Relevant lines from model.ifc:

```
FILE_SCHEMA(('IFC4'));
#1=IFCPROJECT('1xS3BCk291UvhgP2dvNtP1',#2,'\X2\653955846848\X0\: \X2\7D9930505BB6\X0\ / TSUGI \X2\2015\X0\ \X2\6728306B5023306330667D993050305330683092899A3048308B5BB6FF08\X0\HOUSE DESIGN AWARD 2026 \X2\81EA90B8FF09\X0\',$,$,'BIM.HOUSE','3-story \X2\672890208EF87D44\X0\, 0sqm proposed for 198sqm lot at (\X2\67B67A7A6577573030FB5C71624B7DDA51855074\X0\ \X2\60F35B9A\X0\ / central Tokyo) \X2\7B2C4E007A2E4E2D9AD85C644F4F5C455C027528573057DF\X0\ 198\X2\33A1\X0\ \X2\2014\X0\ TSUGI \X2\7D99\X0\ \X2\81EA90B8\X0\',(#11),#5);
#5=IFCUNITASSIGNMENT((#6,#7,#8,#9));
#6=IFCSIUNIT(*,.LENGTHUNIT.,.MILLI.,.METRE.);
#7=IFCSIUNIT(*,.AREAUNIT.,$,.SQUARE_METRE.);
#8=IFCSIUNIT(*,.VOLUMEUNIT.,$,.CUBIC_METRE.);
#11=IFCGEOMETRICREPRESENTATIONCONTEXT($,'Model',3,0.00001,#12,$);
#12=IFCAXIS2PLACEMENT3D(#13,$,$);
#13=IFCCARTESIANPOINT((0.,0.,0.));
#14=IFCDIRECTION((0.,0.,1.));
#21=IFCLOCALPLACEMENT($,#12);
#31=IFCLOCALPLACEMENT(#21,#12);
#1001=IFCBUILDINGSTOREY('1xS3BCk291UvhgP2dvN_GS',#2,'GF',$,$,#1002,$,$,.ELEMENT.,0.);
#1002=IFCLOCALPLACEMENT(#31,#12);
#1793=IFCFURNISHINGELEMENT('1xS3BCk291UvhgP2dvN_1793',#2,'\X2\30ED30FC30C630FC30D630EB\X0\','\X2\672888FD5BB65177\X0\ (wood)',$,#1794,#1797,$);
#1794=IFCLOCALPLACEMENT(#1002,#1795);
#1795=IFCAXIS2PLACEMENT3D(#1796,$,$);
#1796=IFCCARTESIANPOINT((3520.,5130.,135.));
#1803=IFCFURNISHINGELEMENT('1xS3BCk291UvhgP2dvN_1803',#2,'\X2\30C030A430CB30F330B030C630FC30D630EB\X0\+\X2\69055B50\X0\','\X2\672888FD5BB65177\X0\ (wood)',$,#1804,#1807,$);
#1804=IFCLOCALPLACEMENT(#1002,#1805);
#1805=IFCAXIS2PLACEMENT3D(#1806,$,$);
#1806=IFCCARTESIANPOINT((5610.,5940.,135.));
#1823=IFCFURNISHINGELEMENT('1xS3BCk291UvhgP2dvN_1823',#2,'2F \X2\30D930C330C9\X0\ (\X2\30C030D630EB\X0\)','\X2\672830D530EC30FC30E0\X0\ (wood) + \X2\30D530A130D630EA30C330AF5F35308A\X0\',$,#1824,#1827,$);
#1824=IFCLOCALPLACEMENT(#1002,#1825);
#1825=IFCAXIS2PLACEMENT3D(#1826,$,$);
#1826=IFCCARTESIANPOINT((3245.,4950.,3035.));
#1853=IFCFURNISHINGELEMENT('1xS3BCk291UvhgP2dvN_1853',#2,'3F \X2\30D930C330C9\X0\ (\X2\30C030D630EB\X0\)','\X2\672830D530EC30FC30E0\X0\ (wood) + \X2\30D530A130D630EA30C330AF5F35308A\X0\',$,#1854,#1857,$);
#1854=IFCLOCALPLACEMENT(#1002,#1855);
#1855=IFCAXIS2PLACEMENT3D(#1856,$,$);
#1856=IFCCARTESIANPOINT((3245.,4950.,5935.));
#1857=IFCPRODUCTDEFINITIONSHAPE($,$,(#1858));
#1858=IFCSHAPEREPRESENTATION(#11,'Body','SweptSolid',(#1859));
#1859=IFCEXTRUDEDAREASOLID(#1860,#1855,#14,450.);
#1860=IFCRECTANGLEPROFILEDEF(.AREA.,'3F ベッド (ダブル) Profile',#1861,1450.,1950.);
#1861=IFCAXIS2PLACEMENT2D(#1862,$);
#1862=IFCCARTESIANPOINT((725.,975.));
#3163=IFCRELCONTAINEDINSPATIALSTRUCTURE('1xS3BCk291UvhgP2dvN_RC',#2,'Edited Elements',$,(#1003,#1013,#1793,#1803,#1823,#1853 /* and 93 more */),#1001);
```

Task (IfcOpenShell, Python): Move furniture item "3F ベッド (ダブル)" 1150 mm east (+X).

```python
import ifcopenshell
import ifcopenshell.api.geometry
import ifcopenshell.util.placement

model = ifcopenshell.open("model.ifc")

item = model.by_guid("1xS3BCk291UvhgP2dvN_1853")
matrix = ifcopenshell.util.placement.get_local_placement(item.ObjectPlacement)
matrix[0, 3] += 1150.0
ifcopenshell.api.geometry.edit_object_placement(model, product=item, matrix=matrix, is_si=False)

print(ifcopenshell.util.placement.get_local_placement(item.ObjectPlacement).round(3) + 0.0)

model.write("model_edited.ifc")
```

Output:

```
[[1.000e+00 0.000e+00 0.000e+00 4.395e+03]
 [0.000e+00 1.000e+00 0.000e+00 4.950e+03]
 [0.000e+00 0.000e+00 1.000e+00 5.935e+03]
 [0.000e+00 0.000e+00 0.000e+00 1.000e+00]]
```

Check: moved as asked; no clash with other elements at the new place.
